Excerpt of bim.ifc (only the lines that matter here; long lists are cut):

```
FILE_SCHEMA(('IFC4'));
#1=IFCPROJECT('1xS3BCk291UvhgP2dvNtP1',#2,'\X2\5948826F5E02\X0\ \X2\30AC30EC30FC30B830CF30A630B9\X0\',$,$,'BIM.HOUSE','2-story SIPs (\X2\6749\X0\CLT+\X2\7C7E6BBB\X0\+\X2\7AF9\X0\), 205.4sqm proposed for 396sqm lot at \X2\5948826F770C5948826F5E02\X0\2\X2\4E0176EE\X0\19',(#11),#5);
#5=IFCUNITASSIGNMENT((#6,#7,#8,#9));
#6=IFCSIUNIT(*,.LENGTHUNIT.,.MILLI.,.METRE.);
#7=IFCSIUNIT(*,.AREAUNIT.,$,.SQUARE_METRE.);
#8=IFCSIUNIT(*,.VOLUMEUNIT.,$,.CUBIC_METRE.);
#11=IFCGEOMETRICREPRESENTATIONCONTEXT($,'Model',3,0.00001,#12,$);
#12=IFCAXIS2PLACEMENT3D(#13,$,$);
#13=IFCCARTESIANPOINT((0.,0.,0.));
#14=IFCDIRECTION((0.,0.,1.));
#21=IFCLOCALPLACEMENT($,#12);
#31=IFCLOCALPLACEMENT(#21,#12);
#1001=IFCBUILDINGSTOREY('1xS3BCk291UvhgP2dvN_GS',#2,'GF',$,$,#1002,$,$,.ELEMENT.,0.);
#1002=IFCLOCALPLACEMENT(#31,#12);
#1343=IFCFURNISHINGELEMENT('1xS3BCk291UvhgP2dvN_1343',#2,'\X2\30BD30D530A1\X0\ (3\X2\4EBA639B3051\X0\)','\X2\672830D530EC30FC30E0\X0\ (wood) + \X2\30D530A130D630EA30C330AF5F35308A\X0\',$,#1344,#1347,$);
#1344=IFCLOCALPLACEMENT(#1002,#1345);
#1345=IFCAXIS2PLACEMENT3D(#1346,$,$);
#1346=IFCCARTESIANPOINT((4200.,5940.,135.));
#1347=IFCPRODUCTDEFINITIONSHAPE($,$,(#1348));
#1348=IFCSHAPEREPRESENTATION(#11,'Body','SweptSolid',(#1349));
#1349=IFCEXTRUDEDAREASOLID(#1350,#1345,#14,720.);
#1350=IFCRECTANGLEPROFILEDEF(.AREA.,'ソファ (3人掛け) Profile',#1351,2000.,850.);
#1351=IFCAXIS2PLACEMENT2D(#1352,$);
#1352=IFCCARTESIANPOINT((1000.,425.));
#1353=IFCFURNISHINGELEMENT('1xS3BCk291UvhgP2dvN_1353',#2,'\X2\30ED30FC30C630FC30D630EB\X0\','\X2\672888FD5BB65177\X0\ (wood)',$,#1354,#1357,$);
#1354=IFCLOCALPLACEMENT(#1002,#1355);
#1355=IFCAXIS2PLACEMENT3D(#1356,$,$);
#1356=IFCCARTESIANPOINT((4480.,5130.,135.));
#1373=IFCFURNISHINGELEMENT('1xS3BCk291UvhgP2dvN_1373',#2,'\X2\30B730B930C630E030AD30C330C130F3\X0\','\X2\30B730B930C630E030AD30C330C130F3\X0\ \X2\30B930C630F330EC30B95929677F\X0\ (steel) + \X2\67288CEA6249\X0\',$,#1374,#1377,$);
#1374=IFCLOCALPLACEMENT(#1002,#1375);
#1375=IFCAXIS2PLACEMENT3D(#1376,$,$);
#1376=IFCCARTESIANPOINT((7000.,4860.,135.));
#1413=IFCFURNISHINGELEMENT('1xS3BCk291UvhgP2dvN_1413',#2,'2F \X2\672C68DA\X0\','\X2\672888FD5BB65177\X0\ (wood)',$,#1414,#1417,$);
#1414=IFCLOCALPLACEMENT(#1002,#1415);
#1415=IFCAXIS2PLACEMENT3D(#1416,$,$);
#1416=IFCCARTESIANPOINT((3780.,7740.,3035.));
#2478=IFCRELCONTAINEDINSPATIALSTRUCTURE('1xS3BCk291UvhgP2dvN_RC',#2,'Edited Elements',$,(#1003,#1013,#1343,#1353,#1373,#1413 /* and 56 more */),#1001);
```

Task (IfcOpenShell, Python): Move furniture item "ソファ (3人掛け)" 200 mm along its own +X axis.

```python
import ifcopenshell
import ifcopenshell.api.geometry
import ifcopenshell.util.placement
import ifcopenshell.util.unit

model = ifcopenshell.open("bim.ifc")
unit_scale = ifcopenshell.util.unit.calculate_unit_scale(model)

item = model.by_guid("1xS3BCk291UvhgP2dvN_1343")
matrix = ifcopenshell.util.placement.get_local_placement(item.ObjectPlacement)
matrix[:3, 3] += matrix[:3, 0] * 0.2 / unit_scale
ifcopenshell.api.geometry.edit_object_placement(model, product=item, matrix=matrix, is_si=False)

print(ifcopenshell.util.placement.get_local_placement(item.ObjectPlacement).round(3) + 0.0)

model.write("bim_rev.ifc")
```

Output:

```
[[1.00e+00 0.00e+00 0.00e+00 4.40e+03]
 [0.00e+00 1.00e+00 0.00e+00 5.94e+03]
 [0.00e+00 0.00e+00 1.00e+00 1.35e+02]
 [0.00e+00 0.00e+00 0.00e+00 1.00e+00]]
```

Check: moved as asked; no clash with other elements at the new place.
